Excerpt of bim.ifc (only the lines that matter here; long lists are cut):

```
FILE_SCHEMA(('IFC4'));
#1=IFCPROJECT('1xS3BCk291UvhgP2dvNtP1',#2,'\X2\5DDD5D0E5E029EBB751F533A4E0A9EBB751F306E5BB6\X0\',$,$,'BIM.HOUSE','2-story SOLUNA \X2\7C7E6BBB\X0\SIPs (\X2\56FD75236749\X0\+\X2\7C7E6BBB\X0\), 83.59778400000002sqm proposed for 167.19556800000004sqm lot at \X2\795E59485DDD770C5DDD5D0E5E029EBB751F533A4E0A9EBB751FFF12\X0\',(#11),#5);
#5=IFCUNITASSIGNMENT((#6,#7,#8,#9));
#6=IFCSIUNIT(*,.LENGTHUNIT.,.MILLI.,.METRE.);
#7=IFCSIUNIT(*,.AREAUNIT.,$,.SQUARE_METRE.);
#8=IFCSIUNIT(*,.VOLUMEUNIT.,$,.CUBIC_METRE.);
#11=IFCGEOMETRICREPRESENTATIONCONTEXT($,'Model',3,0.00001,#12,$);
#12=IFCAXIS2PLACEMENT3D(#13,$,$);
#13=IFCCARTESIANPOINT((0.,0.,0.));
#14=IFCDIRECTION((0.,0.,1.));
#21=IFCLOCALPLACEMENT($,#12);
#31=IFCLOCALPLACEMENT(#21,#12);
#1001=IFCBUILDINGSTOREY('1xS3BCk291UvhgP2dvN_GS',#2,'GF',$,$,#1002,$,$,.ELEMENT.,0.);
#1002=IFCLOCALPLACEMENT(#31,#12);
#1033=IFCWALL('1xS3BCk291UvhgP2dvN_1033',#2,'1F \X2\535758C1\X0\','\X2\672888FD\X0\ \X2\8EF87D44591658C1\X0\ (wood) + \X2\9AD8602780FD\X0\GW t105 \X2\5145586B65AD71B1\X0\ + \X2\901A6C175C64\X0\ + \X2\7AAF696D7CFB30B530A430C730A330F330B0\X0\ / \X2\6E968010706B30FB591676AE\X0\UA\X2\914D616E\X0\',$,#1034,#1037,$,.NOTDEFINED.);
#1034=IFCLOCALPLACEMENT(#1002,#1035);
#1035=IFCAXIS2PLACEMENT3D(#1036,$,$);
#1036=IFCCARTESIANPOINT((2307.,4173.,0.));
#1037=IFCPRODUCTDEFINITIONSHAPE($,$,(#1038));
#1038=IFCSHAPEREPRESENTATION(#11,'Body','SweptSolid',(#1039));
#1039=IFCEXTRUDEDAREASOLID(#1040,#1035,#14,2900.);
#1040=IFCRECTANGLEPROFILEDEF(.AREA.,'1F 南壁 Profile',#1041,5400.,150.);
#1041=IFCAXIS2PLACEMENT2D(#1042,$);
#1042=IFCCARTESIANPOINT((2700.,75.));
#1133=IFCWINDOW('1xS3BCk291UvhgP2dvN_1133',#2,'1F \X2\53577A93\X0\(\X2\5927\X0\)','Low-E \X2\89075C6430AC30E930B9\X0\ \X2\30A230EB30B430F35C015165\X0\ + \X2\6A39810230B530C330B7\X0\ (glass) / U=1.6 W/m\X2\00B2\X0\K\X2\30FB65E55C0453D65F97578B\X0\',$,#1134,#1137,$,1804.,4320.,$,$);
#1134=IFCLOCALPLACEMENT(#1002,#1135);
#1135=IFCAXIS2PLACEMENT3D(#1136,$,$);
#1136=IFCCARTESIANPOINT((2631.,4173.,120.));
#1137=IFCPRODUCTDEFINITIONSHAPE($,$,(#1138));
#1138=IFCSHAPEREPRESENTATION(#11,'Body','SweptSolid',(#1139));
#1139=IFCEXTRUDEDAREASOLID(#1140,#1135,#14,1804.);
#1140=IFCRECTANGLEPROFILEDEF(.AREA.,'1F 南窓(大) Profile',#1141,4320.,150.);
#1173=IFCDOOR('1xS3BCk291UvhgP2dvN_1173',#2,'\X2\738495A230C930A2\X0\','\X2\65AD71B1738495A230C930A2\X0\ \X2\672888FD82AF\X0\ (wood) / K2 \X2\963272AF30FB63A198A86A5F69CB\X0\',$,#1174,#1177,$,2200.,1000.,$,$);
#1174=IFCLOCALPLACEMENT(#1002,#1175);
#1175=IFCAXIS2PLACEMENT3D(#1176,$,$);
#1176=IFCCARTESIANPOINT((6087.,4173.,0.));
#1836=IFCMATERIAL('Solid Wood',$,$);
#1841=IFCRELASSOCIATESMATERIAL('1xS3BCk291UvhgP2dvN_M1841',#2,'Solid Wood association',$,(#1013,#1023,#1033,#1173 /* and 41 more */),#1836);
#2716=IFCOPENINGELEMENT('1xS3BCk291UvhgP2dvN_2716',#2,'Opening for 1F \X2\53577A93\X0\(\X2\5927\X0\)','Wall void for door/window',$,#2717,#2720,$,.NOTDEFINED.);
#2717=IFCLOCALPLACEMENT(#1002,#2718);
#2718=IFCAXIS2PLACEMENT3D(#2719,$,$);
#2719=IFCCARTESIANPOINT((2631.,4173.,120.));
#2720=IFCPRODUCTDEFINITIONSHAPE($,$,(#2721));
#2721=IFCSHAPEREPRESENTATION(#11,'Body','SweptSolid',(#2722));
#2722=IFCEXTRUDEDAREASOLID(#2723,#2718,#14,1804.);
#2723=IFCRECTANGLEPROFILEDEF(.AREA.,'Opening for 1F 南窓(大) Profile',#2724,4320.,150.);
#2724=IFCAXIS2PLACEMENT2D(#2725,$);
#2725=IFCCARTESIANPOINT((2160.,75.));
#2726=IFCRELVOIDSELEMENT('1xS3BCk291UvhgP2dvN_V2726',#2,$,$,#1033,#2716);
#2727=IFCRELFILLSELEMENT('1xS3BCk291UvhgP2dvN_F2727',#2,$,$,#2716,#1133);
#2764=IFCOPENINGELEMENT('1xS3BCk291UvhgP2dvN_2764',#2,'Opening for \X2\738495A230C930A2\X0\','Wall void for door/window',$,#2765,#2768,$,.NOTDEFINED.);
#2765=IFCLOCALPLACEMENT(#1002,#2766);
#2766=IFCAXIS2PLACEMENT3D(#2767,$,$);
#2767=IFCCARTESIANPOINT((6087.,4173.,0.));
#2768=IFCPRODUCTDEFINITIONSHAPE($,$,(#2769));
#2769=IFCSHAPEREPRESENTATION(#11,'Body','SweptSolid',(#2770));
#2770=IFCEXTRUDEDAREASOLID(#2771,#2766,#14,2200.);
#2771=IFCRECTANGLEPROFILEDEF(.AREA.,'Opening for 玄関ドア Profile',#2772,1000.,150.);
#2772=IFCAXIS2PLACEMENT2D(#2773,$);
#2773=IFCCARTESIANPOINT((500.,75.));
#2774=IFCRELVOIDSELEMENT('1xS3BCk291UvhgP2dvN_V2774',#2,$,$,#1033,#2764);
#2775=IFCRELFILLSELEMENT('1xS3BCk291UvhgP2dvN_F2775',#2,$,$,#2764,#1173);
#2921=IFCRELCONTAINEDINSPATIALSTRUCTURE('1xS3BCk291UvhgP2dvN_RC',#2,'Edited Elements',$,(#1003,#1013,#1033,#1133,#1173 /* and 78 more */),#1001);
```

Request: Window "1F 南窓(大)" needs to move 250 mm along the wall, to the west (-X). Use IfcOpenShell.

```python
import ifcopenshell
import ifcopenshell.api.geometry
import ifcopenshell.util.placement

model = ifcopenshell.open("bim.ifc")

window = model.by_guid("1xS3BCk291UvhgP2dvN_1133")
opening = window.FillsVoids[0].RelatingOpeningElement
wall = opening.VoidsElements[0].RelatingBuildingElement

wall_matrix = ifcopenshell.util.placement.get_local_placement(wall.ObjectPlacement)
shift = wall_matrix[:3, 0] * -250.0
before = ifcopenshell.util.placement.get_local_placement(window.ObjectPlacement)[:3, 3].copy()

# The window is not placed relative to its opening, so move both.
for product in (opening, window):
    matrix = ifcopenshell.util.placement.get_local_placement(product.ObjectPlacement)
    matrix[:3, 3] += shift
    ifcopenshell.api.geometry.edit_object_placement(model, product=product, matrix=matrix, is_si=False)

after = ifcopenshell.util.placement.get_local_placement(window.ObjectPlacement)[:3, 3]
print("window moved by", (after - before).round(3) + 0.0)

model.write("bim_v2.ifc")
```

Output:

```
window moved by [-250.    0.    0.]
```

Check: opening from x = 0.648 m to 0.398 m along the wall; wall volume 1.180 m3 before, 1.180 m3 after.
